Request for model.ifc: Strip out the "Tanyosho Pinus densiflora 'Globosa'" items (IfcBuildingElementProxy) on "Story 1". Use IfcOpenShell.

First a look at what the model holds.

```python
import ifcopenshell
import ifcopenshell.util.element

model = ifcopenshell.open("model.ifc")
print(model.schema)
storey = next(s for s in model.by_type("IfcBuildingStorey") if s.Name == "Story 1")
proxies = [e for e in ifcopenshell.util.element.get_decomposition(storey) if e.is_a("IfcBuildingElementProxy")]
seen = {}
for e in proxies:
    element_type = ifcopenshell.util.element.get_type(e)
    name = element_type.Name if element_type not in (None, e) else None
    seen[name] = seen.get(name, 0) + 1
for name, count in sorted(seen.items(), key=str):
    print(count, "x", name)
```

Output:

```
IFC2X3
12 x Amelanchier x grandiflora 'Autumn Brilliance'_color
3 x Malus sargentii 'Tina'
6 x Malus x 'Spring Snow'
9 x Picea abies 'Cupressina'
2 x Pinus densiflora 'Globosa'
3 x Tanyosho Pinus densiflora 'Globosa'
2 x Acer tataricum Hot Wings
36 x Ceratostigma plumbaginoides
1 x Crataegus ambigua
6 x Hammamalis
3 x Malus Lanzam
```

```python
import ifcopenshell
import ifcopenshell.api.root
import ifcopenshell.util.element

model = ifcopenshell.open("model.ifc")

storey = next(s for s in model.by_type("IfcBuildingStorey") if s.Name == "Story 1")
proxies = [e for e in ifcopenshell.util.element.get_decomposition(storey) if e.is_a("IfcBuildingElementProxy")]
targets = [e for e in proxies if (t := ifcopenshell.util.element.get_type(e)) not in (None, e) and t.Name == "Tanyosho Pinus densiflora 'Globosa'"]

for e in targets:
    ifcopenshell.api.root.remove_product(model, product=e)
print(len(targets), "removed")

model.write("model_edited.ifc")
```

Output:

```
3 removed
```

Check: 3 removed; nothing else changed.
